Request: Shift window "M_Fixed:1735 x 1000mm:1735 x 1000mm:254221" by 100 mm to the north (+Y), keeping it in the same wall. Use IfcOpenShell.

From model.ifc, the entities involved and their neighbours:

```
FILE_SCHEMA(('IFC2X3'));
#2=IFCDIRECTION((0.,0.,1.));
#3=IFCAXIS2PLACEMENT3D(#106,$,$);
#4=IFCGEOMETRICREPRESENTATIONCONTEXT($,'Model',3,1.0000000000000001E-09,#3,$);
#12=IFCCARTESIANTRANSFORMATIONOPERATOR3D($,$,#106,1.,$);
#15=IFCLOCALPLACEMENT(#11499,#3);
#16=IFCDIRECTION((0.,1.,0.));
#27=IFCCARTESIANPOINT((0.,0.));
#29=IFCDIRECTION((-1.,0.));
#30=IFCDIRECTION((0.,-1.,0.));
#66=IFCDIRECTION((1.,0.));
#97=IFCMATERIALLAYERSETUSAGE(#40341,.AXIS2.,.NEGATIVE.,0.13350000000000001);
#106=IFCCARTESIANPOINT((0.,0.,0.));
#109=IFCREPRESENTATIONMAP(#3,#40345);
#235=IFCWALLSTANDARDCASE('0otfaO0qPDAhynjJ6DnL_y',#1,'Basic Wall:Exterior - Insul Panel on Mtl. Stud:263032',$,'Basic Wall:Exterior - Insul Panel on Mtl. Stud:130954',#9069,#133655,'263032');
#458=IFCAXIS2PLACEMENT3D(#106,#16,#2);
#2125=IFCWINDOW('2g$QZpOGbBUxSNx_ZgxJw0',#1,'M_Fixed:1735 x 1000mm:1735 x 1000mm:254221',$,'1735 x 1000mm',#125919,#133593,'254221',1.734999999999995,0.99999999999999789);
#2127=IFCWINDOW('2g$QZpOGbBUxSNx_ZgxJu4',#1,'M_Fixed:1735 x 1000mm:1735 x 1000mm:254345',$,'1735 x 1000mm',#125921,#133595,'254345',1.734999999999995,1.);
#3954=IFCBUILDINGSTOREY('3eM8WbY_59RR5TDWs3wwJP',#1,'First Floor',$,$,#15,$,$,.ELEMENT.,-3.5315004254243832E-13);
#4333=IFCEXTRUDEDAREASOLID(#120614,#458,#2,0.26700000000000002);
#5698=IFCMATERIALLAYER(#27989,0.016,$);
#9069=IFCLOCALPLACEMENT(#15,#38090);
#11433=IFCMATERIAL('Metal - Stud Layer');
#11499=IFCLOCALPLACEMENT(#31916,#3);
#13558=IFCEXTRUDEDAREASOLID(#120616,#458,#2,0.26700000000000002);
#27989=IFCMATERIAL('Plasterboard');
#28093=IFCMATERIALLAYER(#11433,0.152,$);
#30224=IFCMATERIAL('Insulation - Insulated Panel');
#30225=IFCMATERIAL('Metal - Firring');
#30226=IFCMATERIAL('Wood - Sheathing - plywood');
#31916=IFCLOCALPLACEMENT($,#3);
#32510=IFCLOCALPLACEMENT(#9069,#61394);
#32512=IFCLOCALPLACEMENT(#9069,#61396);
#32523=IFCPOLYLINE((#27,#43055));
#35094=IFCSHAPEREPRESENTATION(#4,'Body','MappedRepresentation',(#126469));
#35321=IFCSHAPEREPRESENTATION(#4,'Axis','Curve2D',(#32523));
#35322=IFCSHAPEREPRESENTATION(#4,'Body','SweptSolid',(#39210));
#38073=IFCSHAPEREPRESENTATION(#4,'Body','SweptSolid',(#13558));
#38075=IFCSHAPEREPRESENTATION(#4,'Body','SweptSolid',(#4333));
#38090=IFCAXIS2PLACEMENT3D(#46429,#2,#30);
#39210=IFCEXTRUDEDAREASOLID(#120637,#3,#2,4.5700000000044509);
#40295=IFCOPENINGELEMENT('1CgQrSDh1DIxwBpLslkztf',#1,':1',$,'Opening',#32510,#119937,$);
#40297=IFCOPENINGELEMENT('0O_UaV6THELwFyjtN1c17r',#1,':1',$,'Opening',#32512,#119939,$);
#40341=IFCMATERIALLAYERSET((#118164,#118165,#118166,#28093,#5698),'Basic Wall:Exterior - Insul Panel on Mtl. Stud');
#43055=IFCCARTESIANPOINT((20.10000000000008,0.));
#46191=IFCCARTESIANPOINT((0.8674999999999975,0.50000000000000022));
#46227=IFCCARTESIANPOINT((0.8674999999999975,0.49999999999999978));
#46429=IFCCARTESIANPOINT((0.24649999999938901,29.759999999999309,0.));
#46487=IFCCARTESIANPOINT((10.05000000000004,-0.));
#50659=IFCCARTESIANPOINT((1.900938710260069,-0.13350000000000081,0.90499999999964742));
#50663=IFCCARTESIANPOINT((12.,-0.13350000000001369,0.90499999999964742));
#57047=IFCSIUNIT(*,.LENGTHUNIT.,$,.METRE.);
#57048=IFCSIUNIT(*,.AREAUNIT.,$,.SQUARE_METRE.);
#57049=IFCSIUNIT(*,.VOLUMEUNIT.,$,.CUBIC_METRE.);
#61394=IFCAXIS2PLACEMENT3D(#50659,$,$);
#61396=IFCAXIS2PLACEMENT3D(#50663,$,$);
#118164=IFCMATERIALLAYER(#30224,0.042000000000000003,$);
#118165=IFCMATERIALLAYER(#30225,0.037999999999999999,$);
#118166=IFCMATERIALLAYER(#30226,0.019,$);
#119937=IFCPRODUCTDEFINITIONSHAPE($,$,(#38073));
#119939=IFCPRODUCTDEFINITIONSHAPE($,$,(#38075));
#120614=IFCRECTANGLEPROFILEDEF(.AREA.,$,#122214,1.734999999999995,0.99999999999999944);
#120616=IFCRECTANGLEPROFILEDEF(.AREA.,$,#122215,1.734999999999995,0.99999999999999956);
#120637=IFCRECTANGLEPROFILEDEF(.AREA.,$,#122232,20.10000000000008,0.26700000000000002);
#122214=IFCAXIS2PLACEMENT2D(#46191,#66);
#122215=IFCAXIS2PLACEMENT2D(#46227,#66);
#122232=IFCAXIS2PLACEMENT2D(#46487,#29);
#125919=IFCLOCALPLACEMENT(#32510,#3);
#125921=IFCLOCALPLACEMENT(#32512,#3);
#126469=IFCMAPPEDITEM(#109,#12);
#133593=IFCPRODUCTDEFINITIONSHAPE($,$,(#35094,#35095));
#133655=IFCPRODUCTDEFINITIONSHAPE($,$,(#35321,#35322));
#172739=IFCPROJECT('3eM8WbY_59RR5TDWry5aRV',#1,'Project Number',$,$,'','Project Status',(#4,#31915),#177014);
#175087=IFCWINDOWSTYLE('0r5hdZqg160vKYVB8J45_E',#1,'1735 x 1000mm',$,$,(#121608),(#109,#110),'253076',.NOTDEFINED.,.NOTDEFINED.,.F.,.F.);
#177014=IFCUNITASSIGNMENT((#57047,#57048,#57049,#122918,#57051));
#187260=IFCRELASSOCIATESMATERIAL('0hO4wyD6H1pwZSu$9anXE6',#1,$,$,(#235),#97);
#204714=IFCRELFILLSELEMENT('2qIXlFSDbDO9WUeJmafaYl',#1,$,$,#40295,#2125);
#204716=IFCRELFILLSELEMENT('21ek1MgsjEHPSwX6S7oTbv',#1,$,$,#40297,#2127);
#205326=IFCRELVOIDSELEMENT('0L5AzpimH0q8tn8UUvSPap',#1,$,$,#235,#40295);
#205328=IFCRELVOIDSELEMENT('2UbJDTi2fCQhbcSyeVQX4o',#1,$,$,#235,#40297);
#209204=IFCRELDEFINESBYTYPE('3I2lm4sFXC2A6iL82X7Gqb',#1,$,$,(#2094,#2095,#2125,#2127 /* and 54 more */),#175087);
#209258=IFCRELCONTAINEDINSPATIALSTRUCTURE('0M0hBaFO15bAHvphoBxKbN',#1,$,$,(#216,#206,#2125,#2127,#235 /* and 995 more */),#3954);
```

```python
import ifcopenshell
import ifcopenshell.api.geometry
import ifcopenshell.util.placement

model = ifcopenshell.open("model.ifc")

window = model.by_id(2125)
opening = window.FillsVoids[0].RelatingOpeningElement
wall = opening.VoidsElements[0].RelatingBuildingElement

wall_matrix = ifcopenshell.util.placement.get_local_placement(wall.ObjectPlacement)
shift = wall_matrix[:3, 0] * -0.1
before = ifcopenshell.util.placement.get_local_placement(window.ObjectPlacement)[:3, 3].copy()

# The window is placed relative to its opening, so it follows when the opening moves.
matrix = ifcopenshell.util.placement.get_local_placement(opening.ObjectPlacement)
matrix[:3, 3] += shift
ifcopenshell.api.geometry.edit_object_placement(
    model, product=opening, matrix=matrix, is_si=False, should_transform_children=True
)

after = ifcopenshell.util.placement.get_local_placement(window.ObjectPlacement)[:3, 3]
print("window moved by", (after - before).round(3) + 0.0)

model.write("model_edited.ifc")
```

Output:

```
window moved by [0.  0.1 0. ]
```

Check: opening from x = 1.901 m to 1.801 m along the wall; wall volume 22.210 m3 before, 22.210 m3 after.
